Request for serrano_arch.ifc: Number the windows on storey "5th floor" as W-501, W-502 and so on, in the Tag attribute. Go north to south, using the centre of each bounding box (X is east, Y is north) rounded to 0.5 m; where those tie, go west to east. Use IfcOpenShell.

First a look at what the model holds.

```python
import ifcopenshell
import ifcopenshell.util.element
import ifcopenshell.util.placement

model = ifcopenshell.open("serrano_arch.ifc")
print(model.schema)
storey = next(s for s in model.by_type("IfcBuildingStorey") if s.Name == "5th floor")
windows = [e for e in ifcopenshell.util.element.get_decomposition(storey) if e.is_a("IfcWindow")]
for e in sorted(windows, key=lambda e: e.id()):
    origin = ifcopenshell.util.placement.get_local_placement(e.ObjectPlacement)[:3, 3]
    print(e.id(), e.Tag, e.Name, origin.round(2) + 0.0, sep=" | ")
```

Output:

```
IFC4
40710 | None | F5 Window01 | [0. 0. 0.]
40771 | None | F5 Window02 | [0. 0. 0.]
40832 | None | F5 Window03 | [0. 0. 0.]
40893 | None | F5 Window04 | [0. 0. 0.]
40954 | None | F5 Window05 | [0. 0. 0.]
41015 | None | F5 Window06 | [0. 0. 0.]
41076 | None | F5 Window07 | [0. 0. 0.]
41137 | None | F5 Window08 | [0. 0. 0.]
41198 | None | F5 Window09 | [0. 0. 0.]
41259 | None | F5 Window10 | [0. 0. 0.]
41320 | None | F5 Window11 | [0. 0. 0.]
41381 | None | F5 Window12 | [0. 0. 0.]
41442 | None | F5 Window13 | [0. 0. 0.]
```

```python
import ifcopenshell
import ifcopenshell.geom
import ifcopenshell.util.element
import ifcopenshell.util.shape

model = ifcopenshell.open("serrano_arch.ifc")
settings = ifcopenshell.geom.settings()
settings.set("use-world-coords", True)


def centre(element):
    shape = ifcopenshell.geom.create_shape(settings, element)
    return ifcopenshell.util.shape.get_bbox_centroid(shape.geometry)


storey = next(s for s in model.by_type("IfcBuildingStorey") if s.Name == "5th floor")
windows = [e for e in ifcopenshell.util.element.get_decomposition(storey) if e.is_a("IfcWindow")]

# Insertion points can sit at a corner or the storey origin, so sort by the geometry (in metres).
centres = {e: centre(e) for e in windows}
windows.sort(key=lambda e: (-round(centres[e][1] / 0.5), centres[e][0]))

for i, e in enumerate(windows, start=1):
    number = f"W-5{i:02d}"
    e.Tag = number
    print(e.id(), number)

model.write("serrano_arch_edited.ifc")
```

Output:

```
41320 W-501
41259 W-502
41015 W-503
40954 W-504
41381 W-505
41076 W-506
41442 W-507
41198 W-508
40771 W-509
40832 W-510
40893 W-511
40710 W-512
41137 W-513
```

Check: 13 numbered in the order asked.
